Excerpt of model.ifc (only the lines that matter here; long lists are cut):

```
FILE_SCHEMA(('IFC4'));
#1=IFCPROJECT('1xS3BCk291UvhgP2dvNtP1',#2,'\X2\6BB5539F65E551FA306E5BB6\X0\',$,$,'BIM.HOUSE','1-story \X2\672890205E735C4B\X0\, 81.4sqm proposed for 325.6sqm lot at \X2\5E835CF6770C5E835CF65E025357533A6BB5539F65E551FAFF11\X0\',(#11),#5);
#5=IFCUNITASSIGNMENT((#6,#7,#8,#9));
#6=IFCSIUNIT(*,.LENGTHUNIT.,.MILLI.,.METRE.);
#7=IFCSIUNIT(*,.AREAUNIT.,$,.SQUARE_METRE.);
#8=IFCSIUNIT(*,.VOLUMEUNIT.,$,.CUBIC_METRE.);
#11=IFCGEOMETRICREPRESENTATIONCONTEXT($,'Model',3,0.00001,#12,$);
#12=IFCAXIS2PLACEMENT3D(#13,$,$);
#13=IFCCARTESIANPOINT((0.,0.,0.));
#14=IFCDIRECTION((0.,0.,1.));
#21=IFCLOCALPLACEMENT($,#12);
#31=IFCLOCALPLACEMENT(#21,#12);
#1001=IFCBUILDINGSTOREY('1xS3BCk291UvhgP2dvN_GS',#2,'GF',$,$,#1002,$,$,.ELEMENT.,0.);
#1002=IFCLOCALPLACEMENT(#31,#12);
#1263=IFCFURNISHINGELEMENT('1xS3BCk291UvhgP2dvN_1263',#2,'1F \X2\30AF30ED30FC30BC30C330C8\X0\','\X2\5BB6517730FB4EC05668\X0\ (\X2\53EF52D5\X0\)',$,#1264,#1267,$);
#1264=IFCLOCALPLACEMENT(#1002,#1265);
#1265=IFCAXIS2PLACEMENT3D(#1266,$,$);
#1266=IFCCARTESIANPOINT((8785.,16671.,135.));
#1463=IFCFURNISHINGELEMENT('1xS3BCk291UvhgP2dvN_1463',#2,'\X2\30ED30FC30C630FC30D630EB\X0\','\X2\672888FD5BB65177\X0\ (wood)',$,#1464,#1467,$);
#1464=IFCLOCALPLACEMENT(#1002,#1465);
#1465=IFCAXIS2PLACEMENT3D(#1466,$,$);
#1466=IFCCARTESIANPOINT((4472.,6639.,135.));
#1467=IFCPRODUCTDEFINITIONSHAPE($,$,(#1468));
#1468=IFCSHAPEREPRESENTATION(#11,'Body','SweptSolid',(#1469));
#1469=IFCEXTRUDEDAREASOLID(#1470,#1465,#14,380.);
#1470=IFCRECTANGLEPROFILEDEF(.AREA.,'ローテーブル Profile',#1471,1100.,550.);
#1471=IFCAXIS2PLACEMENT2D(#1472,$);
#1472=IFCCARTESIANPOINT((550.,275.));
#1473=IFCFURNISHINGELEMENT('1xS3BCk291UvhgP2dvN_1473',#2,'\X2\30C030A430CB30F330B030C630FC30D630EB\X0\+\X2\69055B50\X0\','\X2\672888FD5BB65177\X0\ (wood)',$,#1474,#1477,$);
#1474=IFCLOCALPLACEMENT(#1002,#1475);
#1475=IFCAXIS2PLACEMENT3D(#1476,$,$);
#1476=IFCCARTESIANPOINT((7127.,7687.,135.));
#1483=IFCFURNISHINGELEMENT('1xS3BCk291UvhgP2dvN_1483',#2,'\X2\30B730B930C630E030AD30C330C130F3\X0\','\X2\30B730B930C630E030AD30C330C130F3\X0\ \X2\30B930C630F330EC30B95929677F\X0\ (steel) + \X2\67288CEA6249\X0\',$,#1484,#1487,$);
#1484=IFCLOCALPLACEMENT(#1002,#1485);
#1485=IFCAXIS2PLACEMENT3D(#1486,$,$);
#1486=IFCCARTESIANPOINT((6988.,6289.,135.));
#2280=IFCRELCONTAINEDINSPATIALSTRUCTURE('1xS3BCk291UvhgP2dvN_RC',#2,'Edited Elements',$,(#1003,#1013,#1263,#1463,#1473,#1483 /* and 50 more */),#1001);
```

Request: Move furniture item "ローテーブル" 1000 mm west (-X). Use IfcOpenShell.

```python
import ifcopenshell
import ifcopenshell.api.geometry
import ifcopenshell.util.placement

model = ifcopenshell.open("model.ifc")

item = model.by_guid("1xS3BCk291UvhgP2dvN_1463")
matrix = ifcopenshell.util.placement.get_local_placement(item.ObjectPlacement)
matrix[0, 3] -= 1000.0
ifcopenshell.api.geometry.edit_object_placement(model, product=item, matrix=matrix, is_si=False)

print(ifcopenshell.util.placement.get_local_placement(item.ObjectPlacement).round(3) + 0.0)

model.write("model-out.ifc")
```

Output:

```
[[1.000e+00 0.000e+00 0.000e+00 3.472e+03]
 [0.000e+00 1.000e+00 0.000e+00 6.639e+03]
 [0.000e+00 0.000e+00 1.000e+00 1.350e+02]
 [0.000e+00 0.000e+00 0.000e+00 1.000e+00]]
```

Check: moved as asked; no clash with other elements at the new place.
